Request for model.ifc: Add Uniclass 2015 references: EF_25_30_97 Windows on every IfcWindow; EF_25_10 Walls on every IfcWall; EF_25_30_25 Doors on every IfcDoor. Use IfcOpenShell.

First a look at what the model holds.

```python
import ifcopenshell

model = ifcopenshell.open("model.ifc")
print(model.schema)
print("classifications:", [c.Name for c in model.by_type("IfcClassification")])
for ifc_class in ("IfcDoor", "IfcRoof", "IfcStair", "IfcWall", "IfcWindow"):
    print(ifc_class, len(model.by_type(ifc_class)))
```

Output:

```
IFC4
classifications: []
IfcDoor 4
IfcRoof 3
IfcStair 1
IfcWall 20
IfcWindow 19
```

```python
import ifcopenshell
import ifcopenshell.api.classification

model = ifcopenshell.open("model.ifc")

system = ifcopenshell.api.classification.add_classification(model, classification="Uniclass 2015")

codes = {
    "IfcWindow": ("EF_25_30_97", "Windows"),
    "IfcWall": ("EF_25_10", "Walls"),
    "IfcDoor": ("EF_25_30_25", "Doors"),
}
for ifc_class, (code, name) in codes.items():
    products = model.by_type(ifc_class)
    ifcopenshell.api.classification.add_reference(
        model, products=products, classification=system, identification=code, name=name
    )
    print(code, len(products))

model.write("model-out.ifc")
```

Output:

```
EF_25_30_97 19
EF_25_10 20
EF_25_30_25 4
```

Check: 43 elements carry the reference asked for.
